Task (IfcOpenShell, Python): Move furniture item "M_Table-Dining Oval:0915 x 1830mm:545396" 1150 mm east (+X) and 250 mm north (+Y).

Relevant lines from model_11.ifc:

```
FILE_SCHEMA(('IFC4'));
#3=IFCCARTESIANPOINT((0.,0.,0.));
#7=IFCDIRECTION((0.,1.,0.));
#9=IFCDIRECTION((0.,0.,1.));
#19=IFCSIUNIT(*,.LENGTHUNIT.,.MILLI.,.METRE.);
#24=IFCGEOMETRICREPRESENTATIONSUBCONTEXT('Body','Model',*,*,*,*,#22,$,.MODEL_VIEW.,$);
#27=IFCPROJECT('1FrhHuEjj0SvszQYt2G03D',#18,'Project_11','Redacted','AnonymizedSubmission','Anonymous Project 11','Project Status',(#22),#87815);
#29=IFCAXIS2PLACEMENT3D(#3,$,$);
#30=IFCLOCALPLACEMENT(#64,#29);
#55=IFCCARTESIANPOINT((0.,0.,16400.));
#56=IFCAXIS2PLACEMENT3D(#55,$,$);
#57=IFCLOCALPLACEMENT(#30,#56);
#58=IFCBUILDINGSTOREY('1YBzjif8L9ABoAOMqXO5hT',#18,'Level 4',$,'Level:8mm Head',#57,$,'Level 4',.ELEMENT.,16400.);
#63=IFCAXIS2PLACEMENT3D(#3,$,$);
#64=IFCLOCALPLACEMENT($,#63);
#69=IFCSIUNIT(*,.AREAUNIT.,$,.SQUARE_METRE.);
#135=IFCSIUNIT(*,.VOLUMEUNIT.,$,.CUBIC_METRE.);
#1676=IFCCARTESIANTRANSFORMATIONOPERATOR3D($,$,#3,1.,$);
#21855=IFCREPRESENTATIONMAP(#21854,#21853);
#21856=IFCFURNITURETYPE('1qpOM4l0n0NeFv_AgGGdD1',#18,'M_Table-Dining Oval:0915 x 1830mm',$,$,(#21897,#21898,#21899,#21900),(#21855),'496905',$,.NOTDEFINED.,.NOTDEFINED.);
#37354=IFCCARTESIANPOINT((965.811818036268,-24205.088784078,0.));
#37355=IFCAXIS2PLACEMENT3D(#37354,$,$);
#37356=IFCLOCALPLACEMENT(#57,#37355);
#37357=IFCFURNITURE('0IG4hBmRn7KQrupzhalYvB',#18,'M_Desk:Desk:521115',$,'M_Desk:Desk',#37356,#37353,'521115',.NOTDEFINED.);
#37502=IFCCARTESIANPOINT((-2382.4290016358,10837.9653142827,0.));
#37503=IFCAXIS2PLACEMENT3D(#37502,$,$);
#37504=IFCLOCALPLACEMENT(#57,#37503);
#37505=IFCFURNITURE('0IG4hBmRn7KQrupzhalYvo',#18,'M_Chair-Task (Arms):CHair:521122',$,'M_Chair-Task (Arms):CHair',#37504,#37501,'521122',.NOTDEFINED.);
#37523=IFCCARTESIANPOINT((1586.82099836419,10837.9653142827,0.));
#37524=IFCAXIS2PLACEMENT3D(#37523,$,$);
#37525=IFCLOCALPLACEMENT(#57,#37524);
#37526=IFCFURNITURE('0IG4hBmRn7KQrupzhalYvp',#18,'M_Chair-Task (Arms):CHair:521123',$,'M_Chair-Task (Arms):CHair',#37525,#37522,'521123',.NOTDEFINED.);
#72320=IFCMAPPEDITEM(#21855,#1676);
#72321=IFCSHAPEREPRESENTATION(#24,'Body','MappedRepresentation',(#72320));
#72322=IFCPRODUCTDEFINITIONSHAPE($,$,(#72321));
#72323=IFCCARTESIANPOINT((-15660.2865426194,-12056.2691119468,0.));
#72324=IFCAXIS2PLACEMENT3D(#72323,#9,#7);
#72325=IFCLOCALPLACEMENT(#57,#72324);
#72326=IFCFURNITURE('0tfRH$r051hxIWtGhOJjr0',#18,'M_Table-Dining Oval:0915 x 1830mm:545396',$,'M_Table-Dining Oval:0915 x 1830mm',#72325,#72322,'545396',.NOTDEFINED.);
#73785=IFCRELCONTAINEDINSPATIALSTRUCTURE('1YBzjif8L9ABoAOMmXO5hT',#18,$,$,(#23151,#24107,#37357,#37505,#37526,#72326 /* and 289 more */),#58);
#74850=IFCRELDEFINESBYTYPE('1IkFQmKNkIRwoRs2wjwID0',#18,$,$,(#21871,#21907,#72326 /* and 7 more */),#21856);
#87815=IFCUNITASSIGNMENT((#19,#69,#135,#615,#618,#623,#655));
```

```python
import ifcopenshell
import ifcopenshell.api.geometry
import ifcopenshell.util.placement
import ifcopenshell.util.unit

model = ifcopenshell.open("model_11.ifc")
unit_scale = ifcopenshell.util.unit.calculate_unit_scale(model)

item = model.by_guid("0tfRH$r051hxIWtGhOJjr0")
matrix = ifcopenshell.util.placement.get_local_placement(item.ObjectPlacement)
matrix[0, 3] += 1.15 / unit_scale
matrix[1, 3] += 0.25 / unit_scale
ifcopenshell.api.geometry.edit_object_placement(model, product=item, matrix=matrix, is_si=False)

print(ifcopenshell.util.placement.get_local_placement(item.ObjectPlacement).round(3) + 0.0)

model.write("model_11_edited.ifc")
```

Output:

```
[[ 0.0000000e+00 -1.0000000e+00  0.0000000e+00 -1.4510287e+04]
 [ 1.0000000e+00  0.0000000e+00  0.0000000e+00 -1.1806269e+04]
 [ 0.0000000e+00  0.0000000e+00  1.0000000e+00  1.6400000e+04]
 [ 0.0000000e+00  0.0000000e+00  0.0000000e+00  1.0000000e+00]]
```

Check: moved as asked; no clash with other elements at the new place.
